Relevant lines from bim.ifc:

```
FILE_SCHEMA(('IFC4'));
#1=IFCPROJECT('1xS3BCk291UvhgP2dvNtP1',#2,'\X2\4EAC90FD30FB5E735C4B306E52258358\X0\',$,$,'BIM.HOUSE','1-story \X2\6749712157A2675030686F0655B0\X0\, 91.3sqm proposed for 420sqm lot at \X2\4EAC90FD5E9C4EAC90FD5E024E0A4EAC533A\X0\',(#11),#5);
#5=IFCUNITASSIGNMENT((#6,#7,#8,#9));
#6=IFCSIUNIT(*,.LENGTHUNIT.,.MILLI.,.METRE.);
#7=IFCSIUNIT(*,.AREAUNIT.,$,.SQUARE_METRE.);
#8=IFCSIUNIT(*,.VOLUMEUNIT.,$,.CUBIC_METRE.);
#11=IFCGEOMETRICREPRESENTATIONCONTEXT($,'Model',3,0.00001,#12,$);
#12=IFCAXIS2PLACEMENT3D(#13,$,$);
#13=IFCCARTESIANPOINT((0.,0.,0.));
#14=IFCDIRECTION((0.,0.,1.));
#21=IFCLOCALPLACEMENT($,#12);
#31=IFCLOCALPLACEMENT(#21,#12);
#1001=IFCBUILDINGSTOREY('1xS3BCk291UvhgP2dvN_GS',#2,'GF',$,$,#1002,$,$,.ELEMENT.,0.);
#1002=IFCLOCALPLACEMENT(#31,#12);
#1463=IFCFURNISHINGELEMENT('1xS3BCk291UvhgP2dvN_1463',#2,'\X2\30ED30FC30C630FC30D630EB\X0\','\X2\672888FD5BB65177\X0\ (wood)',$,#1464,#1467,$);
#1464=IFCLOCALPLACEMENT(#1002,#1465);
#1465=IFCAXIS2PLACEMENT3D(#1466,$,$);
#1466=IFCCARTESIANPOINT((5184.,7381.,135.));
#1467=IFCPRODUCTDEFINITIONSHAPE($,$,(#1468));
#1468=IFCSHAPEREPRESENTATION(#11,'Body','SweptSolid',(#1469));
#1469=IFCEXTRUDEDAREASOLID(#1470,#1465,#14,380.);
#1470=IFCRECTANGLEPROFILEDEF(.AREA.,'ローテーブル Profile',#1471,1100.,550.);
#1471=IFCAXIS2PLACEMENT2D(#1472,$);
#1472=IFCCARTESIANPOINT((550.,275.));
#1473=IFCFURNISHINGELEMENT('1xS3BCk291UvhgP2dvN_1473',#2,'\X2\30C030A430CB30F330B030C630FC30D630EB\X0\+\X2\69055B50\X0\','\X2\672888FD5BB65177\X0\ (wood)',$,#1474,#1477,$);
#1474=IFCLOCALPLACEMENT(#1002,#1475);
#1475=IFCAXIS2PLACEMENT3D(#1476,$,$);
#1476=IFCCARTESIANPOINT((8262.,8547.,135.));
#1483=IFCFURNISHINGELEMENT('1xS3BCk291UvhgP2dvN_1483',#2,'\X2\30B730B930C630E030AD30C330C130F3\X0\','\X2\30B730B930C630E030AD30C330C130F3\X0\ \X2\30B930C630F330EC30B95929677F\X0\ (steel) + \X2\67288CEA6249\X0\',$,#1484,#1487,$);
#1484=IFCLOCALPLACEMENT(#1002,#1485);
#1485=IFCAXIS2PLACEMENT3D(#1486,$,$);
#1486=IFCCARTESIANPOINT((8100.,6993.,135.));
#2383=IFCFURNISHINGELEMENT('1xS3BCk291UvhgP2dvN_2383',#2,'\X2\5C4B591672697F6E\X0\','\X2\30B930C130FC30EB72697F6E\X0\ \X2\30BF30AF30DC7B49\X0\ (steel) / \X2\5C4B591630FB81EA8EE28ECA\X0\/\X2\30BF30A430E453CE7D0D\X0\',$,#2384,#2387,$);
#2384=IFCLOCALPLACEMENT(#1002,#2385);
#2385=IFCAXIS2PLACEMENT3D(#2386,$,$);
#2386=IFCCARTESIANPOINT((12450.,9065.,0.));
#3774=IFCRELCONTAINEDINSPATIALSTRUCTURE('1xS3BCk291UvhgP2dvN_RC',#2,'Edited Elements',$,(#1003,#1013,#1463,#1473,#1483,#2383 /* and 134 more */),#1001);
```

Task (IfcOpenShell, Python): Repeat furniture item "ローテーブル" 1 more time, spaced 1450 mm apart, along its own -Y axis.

```python
import ifcopenshell
import ifcopenshell.api.geometry
import ifcopenshell.api.root
import ifcopenshell.util.element
import ifcopenshell.util.placement
import ifcopenshell.util.unit

model = ifcopenshell.open("bim.ifc")
unit_scale = ifcopenshell.util.unit.calculate_unit_scale(model)


def reuse_history(source, copy):
    """copy_class also copies each property set's owner history, people and application; keep the originals."""
    for rel in copy.IsDefinedBy:
        if rel.is_a("IfcRelDefinesByProperties") and (history := rel.RelatingPropertyDefinition.OwnerHistory):
            rel.RelatingPropertyDefinition.OwnerHistory = source.OwnerHistory
            ifcopenshell.util.element.remove_deep2(model, history)


source = model.by_id(1463)
base = ifcopenshell.util.placement.get_local_placement(source.ObjectPlacement)
step = -base[:3, 1] * 1.45 / unit_scale

for i in range(1, 2):
    copy = ifcopenshell.api.root.copy_class(model, product=source)
    copy.Representation = ifcopenshell.util.element.copy_deep(
        model, source.Representation, exclude=["IfcGeometricRepresentationContext", "IfcRepresentationMap"]
    )
    reuse_history(source, copy)
    matrix = base.copy()
    matrix[:3, 3] += i * step
    print("added at", matrix[:3, 3].round(3) + 0.0)
    ifcopenshell.api.geometry.edit_object_placement(model, product=copy, matrix=matrix, is_si=False)

model.write("bim-out.ifc")
```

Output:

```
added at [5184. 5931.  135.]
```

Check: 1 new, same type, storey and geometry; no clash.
